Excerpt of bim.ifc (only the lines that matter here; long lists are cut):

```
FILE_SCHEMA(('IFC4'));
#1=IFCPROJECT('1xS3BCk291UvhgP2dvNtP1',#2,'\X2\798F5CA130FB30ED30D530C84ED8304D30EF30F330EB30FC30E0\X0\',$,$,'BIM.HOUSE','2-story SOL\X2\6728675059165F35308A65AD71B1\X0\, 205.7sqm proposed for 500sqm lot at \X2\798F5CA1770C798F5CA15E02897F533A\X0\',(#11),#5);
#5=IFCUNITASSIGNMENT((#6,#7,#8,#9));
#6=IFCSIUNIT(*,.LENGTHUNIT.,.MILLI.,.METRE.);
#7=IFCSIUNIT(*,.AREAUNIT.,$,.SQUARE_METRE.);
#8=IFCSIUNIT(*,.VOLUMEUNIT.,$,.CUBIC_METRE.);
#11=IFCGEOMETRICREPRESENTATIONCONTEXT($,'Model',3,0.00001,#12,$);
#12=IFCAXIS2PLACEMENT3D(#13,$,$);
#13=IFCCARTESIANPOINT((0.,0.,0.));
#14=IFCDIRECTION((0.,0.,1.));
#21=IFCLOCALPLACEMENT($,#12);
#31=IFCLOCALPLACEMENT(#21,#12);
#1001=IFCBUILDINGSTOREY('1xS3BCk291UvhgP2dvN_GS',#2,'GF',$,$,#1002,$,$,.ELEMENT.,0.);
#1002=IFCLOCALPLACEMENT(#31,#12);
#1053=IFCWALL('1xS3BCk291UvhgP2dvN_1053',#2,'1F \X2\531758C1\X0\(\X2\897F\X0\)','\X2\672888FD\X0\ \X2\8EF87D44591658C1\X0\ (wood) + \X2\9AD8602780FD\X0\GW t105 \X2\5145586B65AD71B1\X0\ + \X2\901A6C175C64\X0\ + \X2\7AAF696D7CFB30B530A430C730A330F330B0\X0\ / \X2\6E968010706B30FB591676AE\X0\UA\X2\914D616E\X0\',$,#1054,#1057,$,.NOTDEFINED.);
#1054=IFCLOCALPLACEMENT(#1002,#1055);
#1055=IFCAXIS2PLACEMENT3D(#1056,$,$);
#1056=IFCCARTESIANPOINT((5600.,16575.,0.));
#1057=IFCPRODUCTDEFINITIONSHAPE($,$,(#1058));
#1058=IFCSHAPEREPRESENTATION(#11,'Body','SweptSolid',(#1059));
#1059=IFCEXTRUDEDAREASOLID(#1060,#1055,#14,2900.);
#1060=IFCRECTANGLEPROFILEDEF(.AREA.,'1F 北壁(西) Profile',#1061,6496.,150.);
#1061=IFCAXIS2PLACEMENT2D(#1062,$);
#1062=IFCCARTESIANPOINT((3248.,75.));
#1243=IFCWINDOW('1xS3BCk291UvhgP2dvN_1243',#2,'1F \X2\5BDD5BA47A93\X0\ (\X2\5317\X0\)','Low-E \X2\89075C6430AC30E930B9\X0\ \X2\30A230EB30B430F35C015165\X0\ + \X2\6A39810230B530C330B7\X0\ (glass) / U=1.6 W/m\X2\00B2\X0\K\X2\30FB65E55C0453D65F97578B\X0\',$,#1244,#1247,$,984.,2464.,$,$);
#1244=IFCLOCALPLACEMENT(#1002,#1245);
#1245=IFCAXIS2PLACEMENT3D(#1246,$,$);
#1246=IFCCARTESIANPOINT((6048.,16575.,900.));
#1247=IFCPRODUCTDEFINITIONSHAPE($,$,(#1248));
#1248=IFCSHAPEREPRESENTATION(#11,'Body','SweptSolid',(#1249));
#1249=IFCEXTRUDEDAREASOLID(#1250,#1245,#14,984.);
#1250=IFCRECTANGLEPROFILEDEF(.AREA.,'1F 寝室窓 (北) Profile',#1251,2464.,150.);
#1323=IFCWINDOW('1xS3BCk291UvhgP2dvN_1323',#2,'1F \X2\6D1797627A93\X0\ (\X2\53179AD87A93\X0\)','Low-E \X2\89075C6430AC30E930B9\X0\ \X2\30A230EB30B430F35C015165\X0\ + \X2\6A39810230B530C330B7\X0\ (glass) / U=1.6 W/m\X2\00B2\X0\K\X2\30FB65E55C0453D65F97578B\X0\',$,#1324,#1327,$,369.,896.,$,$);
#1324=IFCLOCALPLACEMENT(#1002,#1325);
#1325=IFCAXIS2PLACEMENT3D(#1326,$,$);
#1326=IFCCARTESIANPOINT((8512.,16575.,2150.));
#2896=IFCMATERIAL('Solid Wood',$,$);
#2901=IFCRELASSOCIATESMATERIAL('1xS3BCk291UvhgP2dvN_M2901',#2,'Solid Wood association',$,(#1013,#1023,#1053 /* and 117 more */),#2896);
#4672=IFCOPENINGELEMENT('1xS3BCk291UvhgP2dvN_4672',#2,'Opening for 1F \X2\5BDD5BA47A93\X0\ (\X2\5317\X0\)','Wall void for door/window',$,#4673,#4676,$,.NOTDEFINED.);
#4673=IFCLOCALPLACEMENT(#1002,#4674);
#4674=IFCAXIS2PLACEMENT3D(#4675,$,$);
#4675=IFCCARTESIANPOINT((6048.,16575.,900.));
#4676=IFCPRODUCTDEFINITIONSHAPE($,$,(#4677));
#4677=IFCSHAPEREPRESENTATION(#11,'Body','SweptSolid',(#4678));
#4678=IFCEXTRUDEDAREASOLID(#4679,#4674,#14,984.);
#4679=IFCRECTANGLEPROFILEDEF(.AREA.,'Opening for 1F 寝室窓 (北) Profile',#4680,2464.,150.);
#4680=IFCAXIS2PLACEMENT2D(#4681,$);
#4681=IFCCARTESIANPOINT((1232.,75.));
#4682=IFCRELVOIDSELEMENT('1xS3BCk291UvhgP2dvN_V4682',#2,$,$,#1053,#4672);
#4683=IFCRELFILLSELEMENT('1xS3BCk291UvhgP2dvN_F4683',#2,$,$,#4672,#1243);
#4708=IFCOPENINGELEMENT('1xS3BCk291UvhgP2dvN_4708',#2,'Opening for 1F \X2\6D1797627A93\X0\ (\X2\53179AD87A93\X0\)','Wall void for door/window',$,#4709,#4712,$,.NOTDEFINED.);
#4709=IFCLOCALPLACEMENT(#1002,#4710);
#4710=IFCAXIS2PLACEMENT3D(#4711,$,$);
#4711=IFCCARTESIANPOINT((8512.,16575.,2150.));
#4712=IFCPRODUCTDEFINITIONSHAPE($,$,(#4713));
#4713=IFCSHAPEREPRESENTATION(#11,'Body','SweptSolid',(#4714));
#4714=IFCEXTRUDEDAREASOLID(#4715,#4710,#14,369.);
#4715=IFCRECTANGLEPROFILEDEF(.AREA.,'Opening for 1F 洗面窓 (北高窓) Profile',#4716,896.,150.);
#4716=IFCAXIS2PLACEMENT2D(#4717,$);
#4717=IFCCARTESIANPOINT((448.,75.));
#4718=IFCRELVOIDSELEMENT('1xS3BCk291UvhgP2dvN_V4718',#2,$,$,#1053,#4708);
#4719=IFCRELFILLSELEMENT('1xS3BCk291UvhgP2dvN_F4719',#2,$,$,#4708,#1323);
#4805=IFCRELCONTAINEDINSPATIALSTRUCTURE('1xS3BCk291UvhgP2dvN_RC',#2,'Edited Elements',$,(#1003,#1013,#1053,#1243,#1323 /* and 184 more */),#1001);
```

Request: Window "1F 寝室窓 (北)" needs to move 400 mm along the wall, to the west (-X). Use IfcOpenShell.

```python
import ifcopenshell
import ifcopenshell.api.geometry
import ifcopenshell.util.placement

model = ifcopenshell.open("bim.ifc")

window = model.by_guid("1xS3BCk291UvhgP2dvN_1243")
opening = window.FillsVoids[0].RelatingOpeningElement
wall = opening.VoidsElements[0].RelatingBuildingElement

wall_matrix = ifcopenshell.util.placement.get_local_placement(wall.ObjectPlacement)
shift = wall_matrix[:3, 0] * -400.0
before = ifcopenshell.util.placement.get_local_placement(window.ObjectPlacement)[:3, 3].copy()

# The window is not placed relative to its opening, so move both.
for product in (opening, window):
    matrix = ifcopenshell.util.placement.get_local_placement(product.ObjectPlacement)
    matrix[:3, 3] += shift
    ifcopenshell.api.geometry.edit_object_placement(model, product=product, matrix=matrix, is_si=False)

after = ifcopenshell.util.placement.get_local_placement(window.ObjectPlacement)[:3, 3]
print("window moved by", (after - before).round(3) + 0.0)

model.write("bim_rev.ifc")
```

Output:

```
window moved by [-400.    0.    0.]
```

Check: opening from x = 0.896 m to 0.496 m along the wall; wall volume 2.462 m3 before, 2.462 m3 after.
